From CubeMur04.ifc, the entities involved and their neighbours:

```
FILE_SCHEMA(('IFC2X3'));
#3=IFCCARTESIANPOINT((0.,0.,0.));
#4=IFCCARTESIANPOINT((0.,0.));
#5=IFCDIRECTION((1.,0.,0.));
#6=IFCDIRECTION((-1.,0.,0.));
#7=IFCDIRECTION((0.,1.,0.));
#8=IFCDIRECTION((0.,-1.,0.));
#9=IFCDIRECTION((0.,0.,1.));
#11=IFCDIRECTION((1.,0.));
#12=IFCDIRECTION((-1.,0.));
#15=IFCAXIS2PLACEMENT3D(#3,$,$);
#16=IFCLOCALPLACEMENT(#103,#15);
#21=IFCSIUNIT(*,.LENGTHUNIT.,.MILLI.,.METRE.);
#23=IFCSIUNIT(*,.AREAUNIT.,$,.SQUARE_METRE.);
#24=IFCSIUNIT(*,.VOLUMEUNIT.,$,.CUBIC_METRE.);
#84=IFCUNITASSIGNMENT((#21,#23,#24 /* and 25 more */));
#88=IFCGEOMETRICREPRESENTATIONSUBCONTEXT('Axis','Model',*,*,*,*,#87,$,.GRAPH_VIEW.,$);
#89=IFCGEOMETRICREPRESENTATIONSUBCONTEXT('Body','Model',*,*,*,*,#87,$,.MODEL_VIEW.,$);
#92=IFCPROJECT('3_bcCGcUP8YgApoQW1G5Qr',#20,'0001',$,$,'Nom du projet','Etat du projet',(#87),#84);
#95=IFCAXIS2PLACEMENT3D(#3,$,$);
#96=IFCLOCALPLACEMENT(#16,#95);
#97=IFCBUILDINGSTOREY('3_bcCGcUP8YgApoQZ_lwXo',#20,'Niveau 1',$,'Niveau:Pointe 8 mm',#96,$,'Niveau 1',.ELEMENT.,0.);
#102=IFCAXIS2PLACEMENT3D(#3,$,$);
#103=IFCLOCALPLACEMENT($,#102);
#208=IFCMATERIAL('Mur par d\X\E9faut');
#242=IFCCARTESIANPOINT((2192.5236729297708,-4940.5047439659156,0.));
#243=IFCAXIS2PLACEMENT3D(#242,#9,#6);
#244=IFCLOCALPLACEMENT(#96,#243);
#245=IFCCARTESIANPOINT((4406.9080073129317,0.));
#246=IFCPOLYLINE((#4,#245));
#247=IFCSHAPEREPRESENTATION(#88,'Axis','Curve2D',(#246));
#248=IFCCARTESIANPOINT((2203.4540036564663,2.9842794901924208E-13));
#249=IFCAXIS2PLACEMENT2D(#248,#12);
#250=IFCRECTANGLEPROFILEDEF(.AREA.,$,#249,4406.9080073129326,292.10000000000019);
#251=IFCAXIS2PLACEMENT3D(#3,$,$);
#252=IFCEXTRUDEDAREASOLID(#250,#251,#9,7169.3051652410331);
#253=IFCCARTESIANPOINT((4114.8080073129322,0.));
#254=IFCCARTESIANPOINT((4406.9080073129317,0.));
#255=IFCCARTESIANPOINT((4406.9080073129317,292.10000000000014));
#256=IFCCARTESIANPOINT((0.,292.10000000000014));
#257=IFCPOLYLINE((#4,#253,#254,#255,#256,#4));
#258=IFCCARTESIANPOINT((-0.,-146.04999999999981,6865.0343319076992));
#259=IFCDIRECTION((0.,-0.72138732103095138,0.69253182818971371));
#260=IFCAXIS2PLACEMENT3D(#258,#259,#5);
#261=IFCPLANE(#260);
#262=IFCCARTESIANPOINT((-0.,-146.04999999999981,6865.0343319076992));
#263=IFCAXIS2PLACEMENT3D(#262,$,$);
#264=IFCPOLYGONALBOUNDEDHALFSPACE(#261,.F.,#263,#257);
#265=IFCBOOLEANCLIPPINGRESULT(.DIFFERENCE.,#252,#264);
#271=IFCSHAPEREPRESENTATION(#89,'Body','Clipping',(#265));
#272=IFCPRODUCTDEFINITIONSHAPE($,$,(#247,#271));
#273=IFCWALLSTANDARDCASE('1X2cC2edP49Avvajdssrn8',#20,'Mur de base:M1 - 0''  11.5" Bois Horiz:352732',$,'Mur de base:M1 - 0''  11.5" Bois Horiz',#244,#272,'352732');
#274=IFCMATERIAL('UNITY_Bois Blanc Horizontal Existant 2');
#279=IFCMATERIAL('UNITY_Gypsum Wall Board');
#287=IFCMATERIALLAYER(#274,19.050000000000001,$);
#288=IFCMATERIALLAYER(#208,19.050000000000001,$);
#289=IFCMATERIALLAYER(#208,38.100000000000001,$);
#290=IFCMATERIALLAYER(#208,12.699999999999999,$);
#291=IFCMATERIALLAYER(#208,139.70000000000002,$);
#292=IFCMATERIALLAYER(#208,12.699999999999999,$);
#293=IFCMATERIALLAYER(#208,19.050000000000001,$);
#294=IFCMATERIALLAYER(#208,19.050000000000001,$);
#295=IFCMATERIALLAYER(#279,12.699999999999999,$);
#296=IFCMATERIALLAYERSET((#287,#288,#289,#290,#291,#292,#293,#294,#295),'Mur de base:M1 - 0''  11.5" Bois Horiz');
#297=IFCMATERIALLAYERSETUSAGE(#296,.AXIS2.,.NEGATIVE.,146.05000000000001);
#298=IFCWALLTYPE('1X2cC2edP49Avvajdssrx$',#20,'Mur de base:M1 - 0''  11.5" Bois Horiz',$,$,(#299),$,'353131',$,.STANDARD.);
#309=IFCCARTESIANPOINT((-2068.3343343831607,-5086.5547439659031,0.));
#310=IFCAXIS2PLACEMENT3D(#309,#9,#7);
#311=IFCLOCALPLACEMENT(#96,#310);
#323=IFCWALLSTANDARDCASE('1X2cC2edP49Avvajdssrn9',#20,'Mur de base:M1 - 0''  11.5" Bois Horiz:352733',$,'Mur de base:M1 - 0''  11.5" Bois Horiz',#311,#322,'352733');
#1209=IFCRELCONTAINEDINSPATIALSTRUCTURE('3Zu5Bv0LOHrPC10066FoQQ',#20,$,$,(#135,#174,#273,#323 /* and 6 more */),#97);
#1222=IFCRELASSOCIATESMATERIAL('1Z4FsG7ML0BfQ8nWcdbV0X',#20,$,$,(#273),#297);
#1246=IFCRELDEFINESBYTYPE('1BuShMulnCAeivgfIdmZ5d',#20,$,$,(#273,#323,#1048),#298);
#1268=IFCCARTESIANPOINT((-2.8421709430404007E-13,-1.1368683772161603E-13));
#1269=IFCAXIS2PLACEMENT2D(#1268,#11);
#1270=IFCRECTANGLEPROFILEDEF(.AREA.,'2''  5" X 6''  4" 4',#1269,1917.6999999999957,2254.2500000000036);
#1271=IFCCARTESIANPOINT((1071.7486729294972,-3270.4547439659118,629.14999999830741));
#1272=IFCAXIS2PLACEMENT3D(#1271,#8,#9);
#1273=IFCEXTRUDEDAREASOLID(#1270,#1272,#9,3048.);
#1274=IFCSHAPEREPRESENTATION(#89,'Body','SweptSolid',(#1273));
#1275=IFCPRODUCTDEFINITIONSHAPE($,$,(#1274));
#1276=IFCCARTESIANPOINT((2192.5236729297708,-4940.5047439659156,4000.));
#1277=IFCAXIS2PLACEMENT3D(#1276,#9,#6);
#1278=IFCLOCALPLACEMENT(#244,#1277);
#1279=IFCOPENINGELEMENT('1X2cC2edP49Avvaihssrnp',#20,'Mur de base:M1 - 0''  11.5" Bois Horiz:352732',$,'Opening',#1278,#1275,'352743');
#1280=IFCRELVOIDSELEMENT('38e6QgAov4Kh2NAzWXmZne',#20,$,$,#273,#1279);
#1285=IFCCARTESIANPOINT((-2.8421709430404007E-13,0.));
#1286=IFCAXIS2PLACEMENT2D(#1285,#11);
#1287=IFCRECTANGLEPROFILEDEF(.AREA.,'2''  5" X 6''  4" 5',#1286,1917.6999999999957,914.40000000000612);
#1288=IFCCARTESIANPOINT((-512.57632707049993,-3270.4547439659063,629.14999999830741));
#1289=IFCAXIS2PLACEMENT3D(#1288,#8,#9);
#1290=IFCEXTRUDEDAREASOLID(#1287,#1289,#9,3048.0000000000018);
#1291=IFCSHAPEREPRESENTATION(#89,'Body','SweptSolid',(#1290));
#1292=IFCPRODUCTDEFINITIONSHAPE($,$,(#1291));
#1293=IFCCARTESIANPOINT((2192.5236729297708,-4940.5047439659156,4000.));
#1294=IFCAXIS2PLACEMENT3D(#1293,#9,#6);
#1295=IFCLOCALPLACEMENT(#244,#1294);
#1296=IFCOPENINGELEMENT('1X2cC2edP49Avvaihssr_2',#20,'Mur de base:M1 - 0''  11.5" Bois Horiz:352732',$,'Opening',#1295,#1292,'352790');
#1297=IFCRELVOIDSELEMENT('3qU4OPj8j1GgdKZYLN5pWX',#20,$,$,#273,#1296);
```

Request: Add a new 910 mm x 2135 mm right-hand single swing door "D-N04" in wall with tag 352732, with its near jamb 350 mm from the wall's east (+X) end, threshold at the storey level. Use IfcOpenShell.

```python
import numpy as np
import ifcopenshell
import ifcopenshell.api.feature
import ifcopenshell.api.geometry
import ifcopenshell.api.root
import ifcopenshell.api.spatial
import ifcopenshell.api.type
import ifcopenshell.geom
import ifcopenshell.util.element
import ifcopenshell.util.placement
import ifcopenshell.util.representation
import ifcopenshell.util.shape
import ifcopenshell.util.unit

model = ifcopenshell.open("CubeMur04.ifc")
unit_scale = ifcopenshell.util.unit.calculate_unit_scale(model)
settings = ifcopenshell.geom.settings()


def volume(element):
    """Net volume in cubic metres, openings subtracted."""
    shape = ifcopenshell.geom.create_shape(settings, element)
    return ifcopenshell.util.shape.get_volume(shape.geometry)


wall = model.by_guid("1X2cC2edP49Avvajdssrn8")
storey = ifcopenshell.util.element.get_container(wall, ifc_class="IfcBuildingStorey")
context = ifcopenshell.util.representation.get_context(model, "Model", "Body", "MODEL_VIEW")
before = volume(wall)

width, height, from_end, sill = 0.91, 2.135, 0.35, 0.0  # metres

# The wall runs along its own X axis, and the end named is its -X end.
wall_shape = ifcopenshell.geom.create_shape(settings, wall)
x, y, z = ifcopenshell.util.shape.get_vertices(wall_shape.geometry).T
start = x.min() + from_end
face, thickness = float(y.min()), float(y.max() - y.min())
wall_matrix = ifcopenshell.util.placement.get_local_placement(wall.ObjectPlacement)
level = ifcopenshell.util.placement.get_local_placement(storey.ObjectPlacement)[2, 3]


def in_wall(x, y):
    """Placement at x, y metres in the wall's axes, at sill height."""
    matrix = wall_matrix.copy()
    matrix[:, 3] = wall_matrix @ np.array([x / unit_scale, y / unit_scale, 0.0, 1.0])
    matrix[2, 3] = level + sill / unit_scale
    return matrix


# Opening: a box that overshoots both wall faces by 50 mm.
opening = ifcopenshell.api.root.create_entity(model, ifc_class="IfcOpeningElement")
box = ifcopenshell.api.geometry.add_wall_representation(
    model, context=context, length=width, height=height, thickness=thickness + 0.1
)
ifcopenshell.api.geometry.assign_representation(model, product=opening, representation=box)
ifcopenshell.api.geometry.edit_object_placement(model, product=opening, matrix=in_wall(start, face - 0.05), is_si=False)
ifcopenshell.api.feature.add_feature(model, feature=opening, element=wall)

door = ifcopenshell.api.root.create_entity(model, ifc_class="IfcDoor", name="D-N04")
door.OverallWidth, door.OverallHeight = width / unit_scale, height / unit_scale
body = ifcopenshell.api.geometry.add_door_representation(
    model,
    context=context,
    overall_width=door.OverallWidth,
    overall_height=door.OverallHeight,
    operation_type="SINGLE_SWING_RIGHT",
    lining_properties={"LiningDepth": thickness / unit_scale, "ThresholdDepth": thickness / unit_scale},
)
ifcopenshell.api.geometry.assign_representation(model, product=door, representation=body)
ifcopenshell.api.spatial.assign_container(model, products=[door], relating_structure=storey)
fills = ifcopenshell.api.feature.add_filling(model, opening=opening, element=door)
fills.OwnerHistory = door.OwnerHistory  # required in IFC2X3

# IFC2X3 keeps the operation on the door style.
style = ifcopenshell.api.root.create_entity(model, ifc_class="IfcDoorStyle", name="D-N04")
style.OperationType, style.ConstructionType = "SINGLE_SWING_RIGHT", "NOTDEFINED"
style.ParameterTakesPrecedence = style.Sizeable = False
ifcopenshell.api.type.assign_type(model, related_objects=[door], relating_type=style)

# The lining spans the wall, so the door starts at the wall face.
ifcopenshell.api.geometry.edit_object_placement(model, product=door, matrix=in_wall(start, face), is_si=False)

after = volume(wall)

print(f"wall volume {before:.3f} -> {after:.3f} m3")

model.write("CubeMur04-out.ifc")
```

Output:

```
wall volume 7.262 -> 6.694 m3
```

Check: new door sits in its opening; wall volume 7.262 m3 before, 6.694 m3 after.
